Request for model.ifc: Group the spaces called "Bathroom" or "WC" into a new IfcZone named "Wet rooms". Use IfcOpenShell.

First a look at what the model holds.

```python
import ifcopenshell

model = ifcopenshell.open("model.ifc")
print(model.schema)
seen = {}
for space in model.by_type("IfcSpace"):
    seen[space.LongName] = seen.get(space.LongName, 0) + 1
for name, count in sorted(seen.items(), key=str):
    print(count, "x", name)
print("zones:", [z.Name for z in model.by_type("IfcZone")][:20])
```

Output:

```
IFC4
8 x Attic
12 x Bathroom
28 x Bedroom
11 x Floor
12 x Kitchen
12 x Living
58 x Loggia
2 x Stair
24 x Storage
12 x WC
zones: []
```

```python
import ifcopenshell
import ifcopenshell.api.group
import ifcopenshell.api.root

model = ifcopenshell.open("model.ifc")

names = {"Bathroom", "WC"}
spaces = [s for s in model.by_type("IfcSpace") if s.LongName in names]

zone = ifcopenshell.api.root.create_entity(model, ifc_class="IfcZone", name="Wet rooms")
ifcopenshell.api.group.assign_group(model, products=spaces, group=zone)
print(len(spaces), "spaces in", zone.Name)

model.write("model_edited.ifc")
```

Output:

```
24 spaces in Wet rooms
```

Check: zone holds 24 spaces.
